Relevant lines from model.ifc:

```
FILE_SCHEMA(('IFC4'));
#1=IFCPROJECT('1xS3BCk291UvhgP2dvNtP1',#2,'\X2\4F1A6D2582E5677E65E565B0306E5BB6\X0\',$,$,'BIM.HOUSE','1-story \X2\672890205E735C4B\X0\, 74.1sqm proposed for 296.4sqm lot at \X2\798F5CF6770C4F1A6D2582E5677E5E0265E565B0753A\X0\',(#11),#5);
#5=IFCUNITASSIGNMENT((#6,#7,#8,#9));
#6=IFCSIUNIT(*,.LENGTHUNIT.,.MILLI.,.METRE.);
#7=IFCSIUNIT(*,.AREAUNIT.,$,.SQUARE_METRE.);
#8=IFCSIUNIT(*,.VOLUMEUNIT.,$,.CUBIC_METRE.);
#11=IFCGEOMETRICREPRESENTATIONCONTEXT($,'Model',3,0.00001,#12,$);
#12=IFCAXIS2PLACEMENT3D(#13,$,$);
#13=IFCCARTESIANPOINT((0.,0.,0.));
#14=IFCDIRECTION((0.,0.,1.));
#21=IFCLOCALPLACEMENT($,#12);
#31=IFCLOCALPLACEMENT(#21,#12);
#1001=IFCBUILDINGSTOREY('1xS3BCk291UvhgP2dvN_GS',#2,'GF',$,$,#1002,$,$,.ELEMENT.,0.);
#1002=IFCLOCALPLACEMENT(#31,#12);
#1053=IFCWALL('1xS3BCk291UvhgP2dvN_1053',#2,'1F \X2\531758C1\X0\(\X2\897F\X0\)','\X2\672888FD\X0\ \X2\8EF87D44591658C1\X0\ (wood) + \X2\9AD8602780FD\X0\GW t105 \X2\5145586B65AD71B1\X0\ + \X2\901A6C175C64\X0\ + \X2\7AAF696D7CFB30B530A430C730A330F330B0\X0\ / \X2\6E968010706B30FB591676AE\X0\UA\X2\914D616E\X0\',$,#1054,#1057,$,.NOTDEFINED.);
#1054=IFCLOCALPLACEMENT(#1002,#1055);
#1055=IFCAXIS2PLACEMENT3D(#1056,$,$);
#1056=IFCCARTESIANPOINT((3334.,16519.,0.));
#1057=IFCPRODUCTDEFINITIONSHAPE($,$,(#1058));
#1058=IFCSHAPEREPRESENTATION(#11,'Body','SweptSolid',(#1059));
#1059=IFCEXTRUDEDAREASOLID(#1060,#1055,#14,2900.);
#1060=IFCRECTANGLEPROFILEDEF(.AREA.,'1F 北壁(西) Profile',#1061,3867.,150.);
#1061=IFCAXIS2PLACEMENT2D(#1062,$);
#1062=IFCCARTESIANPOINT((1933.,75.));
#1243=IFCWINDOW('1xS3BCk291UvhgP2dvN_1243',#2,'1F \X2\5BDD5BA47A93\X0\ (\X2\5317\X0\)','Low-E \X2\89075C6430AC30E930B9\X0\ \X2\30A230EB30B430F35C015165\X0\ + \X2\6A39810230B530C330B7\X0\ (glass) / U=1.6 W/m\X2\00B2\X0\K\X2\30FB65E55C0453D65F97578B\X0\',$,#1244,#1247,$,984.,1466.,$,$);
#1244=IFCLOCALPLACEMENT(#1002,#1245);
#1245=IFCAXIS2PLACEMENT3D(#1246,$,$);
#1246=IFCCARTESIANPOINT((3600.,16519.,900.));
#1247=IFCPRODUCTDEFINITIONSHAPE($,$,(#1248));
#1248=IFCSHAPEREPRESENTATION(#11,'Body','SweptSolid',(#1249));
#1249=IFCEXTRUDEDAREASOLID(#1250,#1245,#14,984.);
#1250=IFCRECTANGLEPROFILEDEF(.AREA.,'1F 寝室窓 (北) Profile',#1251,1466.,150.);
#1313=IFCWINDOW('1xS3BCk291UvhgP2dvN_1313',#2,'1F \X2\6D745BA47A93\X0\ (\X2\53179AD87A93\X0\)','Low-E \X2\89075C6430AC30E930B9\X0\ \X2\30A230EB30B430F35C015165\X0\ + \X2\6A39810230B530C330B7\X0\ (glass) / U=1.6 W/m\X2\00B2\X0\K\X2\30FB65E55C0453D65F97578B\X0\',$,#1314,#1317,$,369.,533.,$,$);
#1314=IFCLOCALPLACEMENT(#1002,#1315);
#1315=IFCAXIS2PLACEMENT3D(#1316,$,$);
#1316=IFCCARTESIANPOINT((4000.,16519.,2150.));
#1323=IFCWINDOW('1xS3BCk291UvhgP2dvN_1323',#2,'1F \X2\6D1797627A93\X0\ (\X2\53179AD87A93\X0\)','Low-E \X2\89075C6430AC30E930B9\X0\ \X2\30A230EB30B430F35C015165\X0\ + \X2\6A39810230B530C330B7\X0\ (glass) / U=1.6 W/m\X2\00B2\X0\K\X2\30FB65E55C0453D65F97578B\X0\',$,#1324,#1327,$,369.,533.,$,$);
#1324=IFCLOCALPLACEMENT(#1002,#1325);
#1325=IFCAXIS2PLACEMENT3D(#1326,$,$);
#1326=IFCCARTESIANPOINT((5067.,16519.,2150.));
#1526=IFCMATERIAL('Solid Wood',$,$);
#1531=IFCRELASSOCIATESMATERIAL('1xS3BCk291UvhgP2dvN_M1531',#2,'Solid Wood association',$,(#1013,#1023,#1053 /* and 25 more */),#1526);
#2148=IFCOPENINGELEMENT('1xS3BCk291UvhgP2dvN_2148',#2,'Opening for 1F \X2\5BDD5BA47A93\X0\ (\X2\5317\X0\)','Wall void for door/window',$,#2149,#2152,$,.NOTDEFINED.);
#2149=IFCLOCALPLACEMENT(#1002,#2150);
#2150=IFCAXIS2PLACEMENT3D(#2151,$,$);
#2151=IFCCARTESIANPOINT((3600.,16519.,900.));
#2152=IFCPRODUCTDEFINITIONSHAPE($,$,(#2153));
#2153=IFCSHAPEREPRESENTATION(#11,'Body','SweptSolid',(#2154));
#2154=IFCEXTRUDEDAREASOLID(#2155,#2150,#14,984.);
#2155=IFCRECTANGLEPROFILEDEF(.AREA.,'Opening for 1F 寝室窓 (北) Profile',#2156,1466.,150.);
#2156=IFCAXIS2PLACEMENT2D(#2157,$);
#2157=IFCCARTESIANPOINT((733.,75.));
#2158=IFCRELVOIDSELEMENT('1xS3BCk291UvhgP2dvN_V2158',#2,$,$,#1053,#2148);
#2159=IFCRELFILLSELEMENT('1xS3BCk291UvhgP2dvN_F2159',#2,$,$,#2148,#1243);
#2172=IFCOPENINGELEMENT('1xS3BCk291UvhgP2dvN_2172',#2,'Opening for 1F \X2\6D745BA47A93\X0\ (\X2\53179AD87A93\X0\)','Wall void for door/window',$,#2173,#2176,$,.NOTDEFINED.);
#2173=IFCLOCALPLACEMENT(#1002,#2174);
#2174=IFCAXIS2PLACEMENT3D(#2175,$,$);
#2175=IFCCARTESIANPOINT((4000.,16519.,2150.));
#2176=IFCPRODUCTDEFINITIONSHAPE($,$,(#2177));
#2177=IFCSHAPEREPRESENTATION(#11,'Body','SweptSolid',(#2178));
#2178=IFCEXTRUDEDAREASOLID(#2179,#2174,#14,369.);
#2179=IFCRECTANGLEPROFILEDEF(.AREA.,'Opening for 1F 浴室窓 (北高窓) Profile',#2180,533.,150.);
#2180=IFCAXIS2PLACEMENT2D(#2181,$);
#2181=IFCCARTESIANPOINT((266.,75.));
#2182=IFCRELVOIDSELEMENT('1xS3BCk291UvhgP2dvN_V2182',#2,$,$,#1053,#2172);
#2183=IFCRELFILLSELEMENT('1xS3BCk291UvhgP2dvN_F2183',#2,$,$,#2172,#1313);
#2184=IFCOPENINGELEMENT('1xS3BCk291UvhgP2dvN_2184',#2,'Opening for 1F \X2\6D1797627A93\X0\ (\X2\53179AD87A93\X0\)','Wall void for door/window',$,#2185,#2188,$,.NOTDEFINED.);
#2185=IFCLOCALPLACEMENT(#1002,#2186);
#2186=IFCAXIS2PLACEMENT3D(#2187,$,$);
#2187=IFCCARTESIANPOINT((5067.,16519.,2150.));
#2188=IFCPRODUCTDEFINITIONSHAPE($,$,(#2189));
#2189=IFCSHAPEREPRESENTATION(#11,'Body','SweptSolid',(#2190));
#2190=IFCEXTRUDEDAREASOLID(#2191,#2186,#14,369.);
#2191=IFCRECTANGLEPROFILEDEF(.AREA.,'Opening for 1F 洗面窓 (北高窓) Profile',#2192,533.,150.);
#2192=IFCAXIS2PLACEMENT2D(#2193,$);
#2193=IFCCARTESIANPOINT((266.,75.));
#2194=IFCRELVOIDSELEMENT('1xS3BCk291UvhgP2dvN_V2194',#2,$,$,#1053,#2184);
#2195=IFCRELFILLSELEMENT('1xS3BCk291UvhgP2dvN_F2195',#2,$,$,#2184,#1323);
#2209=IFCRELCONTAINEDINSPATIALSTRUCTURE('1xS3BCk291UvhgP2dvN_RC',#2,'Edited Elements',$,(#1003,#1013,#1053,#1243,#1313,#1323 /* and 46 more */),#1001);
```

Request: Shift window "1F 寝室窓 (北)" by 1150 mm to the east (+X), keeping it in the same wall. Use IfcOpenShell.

```python
import ifcopenshell
import ifcopenshell.api.geometry
import ifcopenshell.util.placement

model = ifcopenshell.open("model.ifc")

window = model.by_guid("1xS3BCk291UvhgP2dvN_1243")
opening = window.FillsVoids[0].RelatingOpeningElement
wall = opening.VoidsElements[0].RelatingBuildingElement

wall_matrix = ifcopenshell.util.placement.get_local_placement(wall.ObjectPlacement)
shift = wall_matrix[:3, 0] * 1150.0
before = ifcopenshell.util.placement.get_local_placement(window.ObjectPlacement)[:3, 3].copy()

# The window is not placed relative to its opening, so move both.
for product in (opening, window):
    matrix = ifcopenshell.util.placement.get_local_placement(product.ObjectPlacement)
    matrix[:3, 3] += shift
    ifcopenshell.api.geometry.edit_object_placement(model, product=product, matrix=matrix, is_si=False)

after = ifcopenshell.util.placement.get_local_placement(window.ObjectPlacement)[:3, 3]
print("window moved by", (after - before).round(3) + 0.0)

model.write("model_updated.ifc")
```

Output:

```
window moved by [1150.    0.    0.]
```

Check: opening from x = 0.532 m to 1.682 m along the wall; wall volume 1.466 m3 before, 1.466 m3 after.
